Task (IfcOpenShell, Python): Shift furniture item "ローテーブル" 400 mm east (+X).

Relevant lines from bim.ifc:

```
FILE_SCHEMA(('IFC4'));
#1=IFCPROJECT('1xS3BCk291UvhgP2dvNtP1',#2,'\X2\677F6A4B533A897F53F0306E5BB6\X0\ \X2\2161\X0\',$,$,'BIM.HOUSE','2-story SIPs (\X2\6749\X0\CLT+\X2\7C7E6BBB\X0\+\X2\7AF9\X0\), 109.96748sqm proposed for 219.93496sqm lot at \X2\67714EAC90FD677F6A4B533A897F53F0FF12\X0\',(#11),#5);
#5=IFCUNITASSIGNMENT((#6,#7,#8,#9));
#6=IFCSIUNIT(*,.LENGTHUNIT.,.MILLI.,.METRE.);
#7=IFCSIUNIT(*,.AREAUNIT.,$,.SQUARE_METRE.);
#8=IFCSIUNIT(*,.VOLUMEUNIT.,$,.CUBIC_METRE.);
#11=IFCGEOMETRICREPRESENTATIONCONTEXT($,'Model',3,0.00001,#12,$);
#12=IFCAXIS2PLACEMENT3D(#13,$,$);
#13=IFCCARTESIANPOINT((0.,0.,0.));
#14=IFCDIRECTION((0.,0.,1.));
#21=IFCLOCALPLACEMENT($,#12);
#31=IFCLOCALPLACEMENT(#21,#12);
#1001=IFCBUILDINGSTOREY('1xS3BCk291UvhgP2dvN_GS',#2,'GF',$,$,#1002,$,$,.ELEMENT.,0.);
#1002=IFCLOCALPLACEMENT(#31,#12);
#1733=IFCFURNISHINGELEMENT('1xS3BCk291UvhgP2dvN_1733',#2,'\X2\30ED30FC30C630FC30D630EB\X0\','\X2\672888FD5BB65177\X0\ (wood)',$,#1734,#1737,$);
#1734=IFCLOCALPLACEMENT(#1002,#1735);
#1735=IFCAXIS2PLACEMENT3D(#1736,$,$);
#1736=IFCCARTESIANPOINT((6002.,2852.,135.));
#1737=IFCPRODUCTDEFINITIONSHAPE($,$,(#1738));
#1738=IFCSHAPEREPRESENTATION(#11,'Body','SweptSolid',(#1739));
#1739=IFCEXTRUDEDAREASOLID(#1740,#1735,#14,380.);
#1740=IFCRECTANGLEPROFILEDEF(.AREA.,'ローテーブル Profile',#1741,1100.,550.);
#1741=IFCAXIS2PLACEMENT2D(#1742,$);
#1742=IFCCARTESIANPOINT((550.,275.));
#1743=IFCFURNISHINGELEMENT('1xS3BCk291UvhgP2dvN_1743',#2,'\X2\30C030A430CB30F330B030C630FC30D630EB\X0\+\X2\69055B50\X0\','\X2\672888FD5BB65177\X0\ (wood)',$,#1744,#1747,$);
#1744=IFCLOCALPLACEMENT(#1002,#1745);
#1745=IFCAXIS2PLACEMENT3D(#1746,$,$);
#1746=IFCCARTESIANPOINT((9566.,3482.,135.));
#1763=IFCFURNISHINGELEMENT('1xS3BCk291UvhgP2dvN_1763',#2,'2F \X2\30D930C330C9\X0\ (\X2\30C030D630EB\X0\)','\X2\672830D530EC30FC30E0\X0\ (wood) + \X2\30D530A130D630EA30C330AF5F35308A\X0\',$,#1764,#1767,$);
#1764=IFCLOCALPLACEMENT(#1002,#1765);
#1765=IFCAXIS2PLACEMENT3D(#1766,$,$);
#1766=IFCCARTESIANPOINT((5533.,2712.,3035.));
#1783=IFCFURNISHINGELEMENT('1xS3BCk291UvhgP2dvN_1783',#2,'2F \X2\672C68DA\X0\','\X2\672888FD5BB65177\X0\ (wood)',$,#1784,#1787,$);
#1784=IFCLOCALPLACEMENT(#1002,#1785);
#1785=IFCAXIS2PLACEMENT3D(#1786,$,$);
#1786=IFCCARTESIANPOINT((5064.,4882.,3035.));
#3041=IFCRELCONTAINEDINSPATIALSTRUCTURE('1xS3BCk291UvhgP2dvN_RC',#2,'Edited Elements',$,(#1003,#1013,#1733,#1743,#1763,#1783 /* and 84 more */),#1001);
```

```python
import ifcopenshell
import ifcopenshell.api.geometry
import ifcopenshell.util.placement
import ifcopenshell.util.unit

model = ifcopenshell.open("bim.ifc")
unit_scale = ifcopenshell.util.unit.calculate_unit_scale(model)

item = model.by_guid("1xS3BCk291UvhgP2dvN_1733")
matrix = ifcopenshell.util.placement.get_local_placement(item.ObjectPlacement)
matrix[0, 3] += 0.4 / unit_scale
ifcopenshell.api.geometry.edit_object_placement(model, product=item, matrix=matrix, is_si=False)

print(ifcopenshell.util.placement.get_local_placement(item.ObjectPlacement).round(3) + 0.0)

model.write("bim_v2.ifc")
```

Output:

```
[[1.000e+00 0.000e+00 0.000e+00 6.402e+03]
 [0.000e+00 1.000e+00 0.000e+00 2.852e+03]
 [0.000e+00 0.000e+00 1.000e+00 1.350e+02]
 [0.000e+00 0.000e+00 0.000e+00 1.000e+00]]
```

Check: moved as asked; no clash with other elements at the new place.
